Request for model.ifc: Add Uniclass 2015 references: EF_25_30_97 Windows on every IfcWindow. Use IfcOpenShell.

First a look at what the model holds.

```python
import ifcopenshell

model = ifcopenshell.open("model.ifc")
print(model.schema)
print("classifications:", [c.Name for c in model.by_type("IfcClassification")])
for ifc_class in ("IfcDoor", "IfcRoof", "IfcStair", "IfcWall", "IfcWindow"):
    print(ifc_class, len(model.by_type(ifc_class)))
```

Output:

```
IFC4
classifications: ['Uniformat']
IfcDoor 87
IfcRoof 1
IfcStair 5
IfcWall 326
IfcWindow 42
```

```python
import ifcopenshell
import ifcopenshell.api.classification

model = ifcopenshell.open("model.ifc")

system = ifcopenshell.api.classification.add_classification(model, classification="Uniclass 2015")

codes = {
    "IfcWindow": ("EF_25_30_97", "Windows"),
}
for ifc_class, (code, name) in codes.items():
    products = model.by_type(ifc_class)
    ifcopenshell.api.classification.add_reference(
        model, products=products, classification=system, identification=code, name=name
    )
    print(code, len(products))

model.write("model_rev.ifc")
```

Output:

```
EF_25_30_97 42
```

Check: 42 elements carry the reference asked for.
